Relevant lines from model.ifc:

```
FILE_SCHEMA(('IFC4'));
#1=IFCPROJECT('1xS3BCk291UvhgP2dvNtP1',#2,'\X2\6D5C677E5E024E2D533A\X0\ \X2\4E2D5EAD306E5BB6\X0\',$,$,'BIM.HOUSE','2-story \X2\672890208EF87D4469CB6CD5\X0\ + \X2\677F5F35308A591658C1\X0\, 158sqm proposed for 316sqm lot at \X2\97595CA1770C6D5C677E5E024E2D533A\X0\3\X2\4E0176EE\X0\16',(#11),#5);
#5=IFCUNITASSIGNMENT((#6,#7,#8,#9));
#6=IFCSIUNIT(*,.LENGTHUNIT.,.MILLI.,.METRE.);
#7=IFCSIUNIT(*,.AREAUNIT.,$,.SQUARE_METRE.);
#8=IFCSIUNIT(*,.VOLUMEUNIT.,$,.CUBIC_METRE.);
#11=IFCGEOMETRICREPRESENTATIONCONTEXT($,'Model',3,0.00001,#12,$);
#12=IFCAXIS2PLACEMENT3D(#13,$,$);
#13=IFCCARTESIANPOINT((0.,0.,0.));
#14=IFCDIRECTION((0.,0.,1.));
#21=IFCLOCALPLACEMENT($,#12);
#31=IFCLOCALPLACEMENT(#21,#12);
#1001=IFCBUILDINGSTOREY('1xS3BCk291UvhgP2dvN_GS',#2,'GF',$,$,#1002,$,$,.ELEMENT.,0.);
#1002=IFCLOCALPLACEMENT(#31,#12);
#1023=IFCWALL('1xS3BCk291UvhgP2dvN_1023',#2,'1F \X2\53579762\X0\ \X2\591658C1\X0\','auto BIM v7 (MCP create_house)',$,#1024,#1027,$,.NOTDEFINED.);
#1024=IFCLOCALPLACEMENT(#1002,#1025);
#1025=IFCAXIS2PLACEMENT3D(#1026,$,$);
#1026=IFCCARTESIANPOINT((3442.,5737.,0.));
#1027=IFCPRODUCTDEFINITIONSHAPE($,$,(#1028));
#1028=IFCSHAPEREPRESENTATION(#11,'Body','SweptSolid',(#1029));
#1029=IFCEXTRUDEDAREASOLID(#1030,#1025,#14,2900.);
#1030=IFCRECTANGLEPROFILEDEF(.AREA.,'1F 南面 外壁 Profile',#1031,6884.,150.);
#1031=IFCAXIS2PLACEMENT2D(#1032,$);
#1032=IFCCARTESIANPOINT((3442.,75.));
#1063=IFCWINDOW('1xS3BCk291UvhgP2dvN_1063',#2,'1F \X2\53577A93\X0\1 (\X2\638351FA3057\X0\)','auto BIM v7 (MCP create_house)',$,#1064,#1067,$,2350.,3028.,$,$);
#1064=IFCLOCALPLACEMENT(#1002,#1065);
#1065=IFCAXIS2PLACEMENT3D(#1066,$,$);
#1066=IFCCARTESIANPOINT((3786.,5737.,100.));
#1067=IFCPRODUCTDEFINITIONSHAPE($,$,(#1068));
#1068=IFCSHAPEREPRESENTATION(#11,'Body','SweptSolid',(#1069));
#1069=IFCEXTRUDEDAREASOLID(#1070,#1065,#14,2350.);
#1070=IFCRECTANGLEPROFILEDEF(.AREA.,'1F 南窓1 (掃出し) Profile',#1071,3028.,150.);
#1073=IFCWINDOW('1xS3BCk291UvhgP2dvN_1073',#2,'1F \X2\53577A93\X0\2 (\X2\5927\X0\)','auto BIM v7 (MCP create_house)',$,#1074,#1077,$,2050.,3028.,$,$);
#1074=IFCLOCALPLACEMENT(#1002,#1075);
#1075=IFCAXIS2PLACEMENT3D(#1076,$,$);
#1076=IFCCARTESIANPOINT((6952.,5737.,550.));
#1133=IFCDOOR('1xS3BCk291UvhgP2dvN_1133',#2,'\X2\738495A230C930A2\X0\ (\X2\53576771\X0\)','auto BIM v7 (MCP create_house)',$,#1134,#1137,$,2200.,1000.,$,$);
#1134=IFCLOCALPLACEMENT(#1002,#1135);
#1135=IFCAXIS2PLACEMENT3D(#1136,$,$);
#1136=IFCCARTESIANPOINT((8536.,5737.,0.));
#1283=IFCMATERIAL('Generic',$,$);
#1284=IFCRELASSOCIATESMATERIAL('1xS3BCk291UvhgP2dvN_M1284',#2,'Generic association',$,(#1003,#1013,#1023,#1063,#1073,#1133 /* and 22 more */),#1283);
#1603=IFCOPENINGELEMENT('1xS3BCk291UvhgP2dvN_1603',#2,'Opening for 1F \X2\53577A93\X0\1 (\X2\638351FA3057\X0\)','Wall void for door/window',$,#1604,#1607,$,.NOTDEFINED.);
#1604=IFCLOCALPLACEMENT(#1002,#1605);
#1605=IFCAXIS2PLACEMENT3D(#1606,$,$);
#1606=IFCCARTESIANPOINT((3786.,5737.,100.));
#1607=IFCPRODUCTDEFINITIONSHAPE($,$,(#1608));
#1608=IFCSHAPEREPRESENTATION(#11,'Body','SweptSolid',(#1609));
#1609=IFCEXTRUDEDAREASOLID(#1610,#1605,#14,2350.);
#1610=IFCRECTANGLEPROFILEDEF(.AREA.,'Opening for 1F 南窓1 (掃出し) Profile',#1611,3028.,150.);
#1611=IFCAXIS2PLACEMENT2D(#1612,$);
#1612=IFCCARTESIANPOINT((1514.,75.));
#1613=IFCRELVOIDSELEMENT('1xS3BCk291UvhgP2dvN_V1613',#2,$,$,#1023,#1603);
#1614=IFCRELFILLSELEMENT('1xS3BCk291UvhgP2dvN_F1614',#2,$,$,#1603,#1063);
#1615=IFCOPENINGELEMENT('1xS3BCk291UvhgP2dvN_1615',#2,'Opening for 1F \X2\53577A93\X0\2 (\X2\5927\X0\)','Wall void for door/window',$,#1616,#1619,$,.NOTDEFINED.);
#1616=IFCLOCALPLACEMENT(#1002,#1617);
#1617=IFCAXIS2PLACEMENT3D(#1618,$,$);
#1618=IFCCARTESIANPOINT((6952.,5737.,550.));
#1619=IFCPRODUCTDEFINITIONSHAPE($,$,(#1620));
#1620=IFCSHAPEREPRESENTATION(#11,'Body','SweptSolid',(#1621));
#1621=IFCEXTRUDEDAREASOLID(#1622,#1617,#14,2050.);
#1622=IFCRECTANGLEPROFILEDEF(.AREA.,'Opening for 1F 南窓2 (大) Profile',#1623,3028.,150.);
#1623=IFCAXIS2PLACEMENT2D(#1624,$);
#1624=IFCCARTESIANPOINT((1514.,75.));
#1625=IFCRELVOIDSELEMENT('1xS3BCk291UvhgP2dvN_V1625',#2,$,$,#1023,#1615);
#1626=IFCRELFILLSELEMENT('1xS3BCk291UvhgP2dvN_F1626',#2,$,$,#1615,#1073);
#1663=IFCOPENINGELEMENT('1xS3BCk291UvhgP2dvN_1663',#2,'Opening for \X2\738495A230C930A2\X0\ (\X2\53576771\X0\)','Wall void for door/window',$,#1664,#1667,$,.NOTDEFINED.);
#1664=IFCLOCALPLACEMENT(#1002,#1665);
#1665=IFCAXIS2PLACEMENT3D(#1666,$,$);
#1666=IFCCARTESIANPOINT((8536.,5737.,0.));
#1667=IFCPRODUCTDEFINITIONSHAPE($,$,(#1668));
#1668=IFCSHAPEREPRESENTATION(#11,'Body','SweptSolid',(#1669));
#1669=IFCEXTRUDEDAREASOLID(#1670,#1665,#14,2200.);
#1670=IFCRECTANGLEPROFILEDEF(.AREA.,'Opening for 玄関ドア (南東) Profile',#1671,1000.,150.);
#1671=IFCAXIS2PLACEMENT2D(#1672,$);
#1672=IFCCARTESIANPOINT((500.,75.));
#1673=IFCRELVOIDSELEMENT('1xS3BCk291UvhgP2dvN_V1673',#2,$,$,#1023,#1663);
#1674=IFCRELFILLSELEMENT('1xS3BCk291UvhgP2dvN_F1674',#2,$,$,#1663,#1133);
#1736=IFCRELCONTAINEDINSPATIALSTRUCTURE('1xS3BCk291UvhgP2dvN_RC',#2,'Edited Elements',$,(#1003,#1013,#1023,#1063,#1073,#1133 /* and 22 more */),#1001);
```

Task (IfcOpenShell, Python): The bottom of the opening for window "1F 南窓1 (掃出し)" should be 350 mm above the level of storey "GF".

```python
import numpy as np
import ifcopenshell
import ifcopenshell.api.geometry
import ifcopenshell.geom
import ifcopenshell.util.element
import ifcopenshell.util.placement
import ifcopenshell.util.shape
import ifcopenshell.util.unit

model = ifcopenshell.open("model.ifc")
unit_scale = ifcopenshell.util.unit.calculate_unit_scale(model)

window = model.by_guid("1xS3BCk291UvhgP2dvN_1063")
opening = window.FillsVoids[0].RelatingOpeningElement
storey = ifcopenshell.util.element.get_container(window, ifc_class="IfcBuildingStorey")
level = ifcopenshell.util.placement.get_local_placement(storey.ObjectPlacement)[2, 3]

# The opening's origin need not be at the sill, so measure its lowest point.
shape = ifcopenshell.geom.create_shape(ifcopenshell.geom.settings(), opening)
bottom = ifcopenshell.util.shape.get_shape_bottom_elevation(shape, shape.geometry) / unit_scale
dz = level + 0.35 / unit_scale - bottom

shift = np.array([0.0, 0.0, dz])
# The window is not placed relative to its opening, so move both.
for product in (opening, window):
    matrix = ifcopenshell.util.placement.get_local_placement(product.ObjectPlacement)
    matrix[:3, 3] += shift
    ifcopenshell.api.geometry.edit_object_placement(model, product=product, matrix=matrix, is_si=False)

print(f"moved by {dz * unit_scale:+.3f} m")

model.write("model_updated.ifc")
```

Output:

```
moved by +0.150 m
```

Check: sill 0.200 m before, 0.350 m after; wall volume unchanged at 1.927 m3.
